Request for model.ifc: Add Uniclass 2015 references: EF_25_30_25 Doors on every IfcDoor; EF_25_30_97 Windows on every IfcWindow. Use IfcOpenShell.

First a look at what the model holds.

```python
import ifcopenshell

model = ifcopenshell.open("model.ifc")
print(model.schema)
print("classifications:", [c.Name for c in model.by_type("IfcClassification")])
for ifc_class in ("IfcDoor", "IfcRoof", "IfcStair", "IfcWall", "IfcWindow"):
    print(ifc_class, len(model.by_type(ifc_class)))
```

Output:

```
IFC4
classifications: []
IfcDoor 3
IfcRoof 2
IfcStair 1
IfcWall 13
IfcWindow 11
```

```python
import ifcopenshell
import ifcopenshell.api.classification

model = ifcopenshell.open("model.ifc")

system = ifcopenshell.api.classification.add_classification(model, classification="Uniclass 2015")

codes = {
    "IfcDoor": ("EF_25_30_25", "Doors"),
    "IfcWindow": ("EF_25_30_97", "Windows"),
}
for ifc_class, (code, name) in codes.items():
    products = model.by_type(ifc_class)
    ifcopenshell.api.classification.add_reference(
        model, products=products, classification=system, identification=code, name=name
    )
    print(code, len(products))

model.write("model-out.ifc")
```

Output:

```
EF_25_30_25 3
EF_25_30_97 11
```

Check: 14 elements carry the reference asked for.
